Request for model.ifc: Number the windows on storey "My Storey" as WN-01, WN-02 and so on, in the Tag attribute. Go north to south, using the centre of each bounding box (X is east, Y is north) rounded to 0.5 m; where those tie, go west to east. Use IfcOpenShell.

First a look at what the model holds.

```python
import ifcopenshell
import ifcopenshell.util.element
import ifcopenshell.util.placement

model = ifcopenshell.open("model.ifc")
print(model.schema)
storey = next(s for s in model.by_type("IfcBuildingStorey") if s.Name == "My Storey")
windows = [e for e in ifcopenshell.util.element.get_decomposition(storey) if e.is_a("IfcWindow")]
for e in sorted(windows, key=lambda e: e.id()):
    origin = ifcopenshell.util.placement.get_local_placement(e.ObjectPlacement)[:3, 3]
    print(e.id(), e.Tag, e.Name, origin.round(2) + 0.0, sep=" | ")
```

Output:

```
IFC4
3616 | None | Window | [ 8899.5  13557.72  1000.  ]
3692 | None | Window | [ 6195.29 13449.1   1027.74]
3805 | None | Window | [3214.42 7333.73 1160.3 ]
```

```python
import ifcopenshell
import ifcopenshell.geom
import ifcopenshell.util.element
import ifcopenshell.util.shape

model = ifcopenshell.open("model.ifc")
settings = ifcopenshell.geom.settings()
settings.set("use-world-coords", True)


def centre(element):
    shape = ifcopenshell.geom.create_shape(settings, element)
    return ifcopenshell.util.shape.get_bbox_centroid(shape.geometry)


storey = next(s for s in model.by_type("IfcBuildingStorey") if s.Name == "My Storey")
windows = [e for e in ifcopenshell.util.element.get_decomposition(storey) if e.is_a("IfcWindow")]

# Insertion points can sit at a corner or the storey origin, so sort by the geometry (in metres).
centres = {e: centre(e) for e in windows}
windows.sort(key=lambda e: (-round(centres[e][1] / 0.5), centres[e][0]))

for i, e in enumerate(windows, start=1):
    number = f"WN-{i:02d}"
    e.Tag = number
    print(e.id(), number)

model.write("model_v2.ifc")
```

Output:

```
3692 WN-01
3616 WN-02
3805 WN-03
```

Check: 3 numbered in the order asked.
